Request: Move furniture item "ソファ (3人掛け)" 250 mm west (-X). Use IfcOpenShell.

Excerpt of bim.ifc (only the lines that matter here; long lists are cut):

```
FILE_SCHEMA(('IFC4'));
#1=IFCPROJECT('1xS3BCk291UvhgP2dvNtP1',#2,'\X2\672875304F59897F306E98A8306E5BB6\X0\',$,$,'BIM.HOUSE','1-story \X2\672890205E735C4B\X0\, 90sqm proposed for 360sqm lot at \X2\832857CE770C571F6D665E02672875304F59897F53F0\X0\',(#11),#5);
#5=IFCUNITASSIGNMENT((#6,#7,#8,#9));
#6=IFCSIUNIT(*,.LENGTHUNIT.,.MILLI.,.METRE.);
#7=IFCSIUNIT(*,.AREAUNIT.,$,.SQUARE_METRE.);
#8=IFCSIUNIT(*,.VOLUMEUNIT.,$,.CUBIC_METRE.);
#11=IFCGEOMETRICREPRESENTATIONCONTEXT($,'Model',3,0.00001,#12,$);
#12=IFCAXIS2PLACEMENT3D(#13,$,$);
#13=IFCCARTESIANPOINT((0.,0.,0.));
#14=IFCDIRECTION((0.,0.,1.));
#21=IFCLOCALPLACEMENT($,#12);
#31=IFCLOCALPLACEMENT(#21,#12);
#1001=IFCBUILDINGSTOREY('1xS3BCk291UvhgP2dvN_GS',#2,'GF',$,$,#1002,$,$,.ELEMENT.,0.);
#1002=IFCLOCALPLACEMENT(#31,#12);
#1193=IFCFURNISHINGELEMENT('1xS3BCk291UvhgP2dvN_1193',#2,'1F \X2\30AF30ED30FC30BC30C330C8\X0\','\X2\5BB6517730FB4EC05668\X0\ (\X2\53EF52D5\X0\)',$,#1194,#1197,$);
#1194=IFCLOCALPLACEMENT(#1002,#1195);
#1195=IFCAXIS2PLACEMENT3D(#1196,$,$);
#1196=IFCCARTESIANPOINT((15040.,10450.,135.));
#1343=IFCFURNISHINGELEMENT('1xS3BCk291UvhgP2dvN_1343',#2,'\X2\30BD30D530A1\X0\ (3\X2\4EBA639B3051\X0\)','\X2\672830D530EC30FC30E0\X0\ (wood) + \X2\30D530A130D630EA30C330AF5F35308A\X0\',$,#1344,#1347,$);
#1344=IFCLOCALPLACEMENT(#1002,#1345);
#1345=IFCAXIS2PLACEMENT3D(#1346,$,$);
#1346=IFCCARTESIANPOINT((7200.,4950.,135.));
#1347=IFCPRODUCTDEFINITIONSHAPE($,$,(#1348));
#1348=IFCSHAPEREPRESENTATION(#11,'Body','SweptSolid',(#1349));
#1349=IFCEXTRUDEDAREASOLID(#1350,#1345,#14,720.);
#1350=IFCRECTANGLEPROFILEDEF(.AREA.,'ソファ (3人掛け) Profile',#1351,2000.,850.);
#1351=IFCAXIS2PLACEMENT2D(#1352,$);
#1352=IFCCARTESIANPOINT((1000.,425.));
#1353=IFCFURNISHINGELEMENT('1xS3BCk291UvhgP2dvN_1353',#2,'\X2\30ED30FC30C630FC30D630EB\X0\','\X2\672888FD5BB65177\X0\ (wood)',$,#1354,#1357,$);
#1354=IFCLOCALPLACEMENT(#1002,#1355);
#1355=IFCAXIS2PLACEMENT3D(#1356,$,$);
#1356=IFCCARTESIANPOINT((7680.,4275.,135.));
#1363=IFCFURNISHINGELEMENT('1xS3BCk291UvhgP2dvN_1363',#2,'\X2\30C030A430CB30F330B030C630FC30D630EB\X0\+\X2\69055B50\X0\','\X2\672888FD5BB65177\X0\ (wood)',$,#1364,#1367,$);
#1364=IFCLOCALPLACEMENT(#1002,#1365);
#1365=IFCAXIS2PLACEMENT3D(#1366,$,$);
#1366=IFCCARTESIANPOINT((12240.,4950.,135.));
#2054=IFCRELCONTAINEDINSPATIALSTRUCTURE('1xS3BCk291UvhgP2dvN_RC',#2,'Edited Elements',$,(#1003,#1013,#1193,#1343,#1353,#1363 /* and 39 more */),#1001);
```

```python
import ifcopenshell
import ifcopenshell.api.geometry
import ifcopenshell.util.placement
import ifcopenshell.util.unit

model = ifcopenshell.open("bim.ifc")
unit_scale = ifcopenshell.util.unit.calculate_unit_scale(model)

item = model.by_guid("1xS3BCk291UvhgP2dvN_1343")
matrix = ifcopenshell.util.placement.get_local_placement(item.ObjectPlacement)
matrix[0, 3] -= 0.25 / unit_scale
ifcopenshell.api.geometry.edit_object_placement(model, product=item, matrix=matrix, is_si=False)

print(ifcopenshell.util.placement.get_local_placement(item.ObjectPlacement).round(3) + 0.0)

model.write("bim-out.ifc")
```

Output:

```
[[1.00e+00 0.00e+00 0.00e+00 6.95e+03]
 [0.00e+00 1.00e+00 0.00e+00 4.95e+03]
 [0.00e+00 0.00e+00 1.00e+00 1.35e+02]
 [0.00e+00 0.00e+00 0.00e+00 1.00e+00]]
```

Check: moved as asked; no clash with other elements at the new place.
